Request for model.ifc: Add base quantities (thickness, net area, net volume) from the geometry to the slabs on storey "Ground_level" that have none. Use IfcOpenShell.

First a look at what the model holds.

```python
import ifcopenshell
import ifcopenshell.util.element
import ifcopenshell.util.unit

model = ifcopenshell.open("model.ifc")
print(model.schema)
for unit_type in ("LENGTHUNIT", "AREAUNIT", "VOLUMEUNIT"):
    print(unit_type, ifcopenshell.util.unit.calculate_unit_scale(model, unit_type))
storey = next(s for s in model.by_type("IfcBuildingStorey") if s.Name == "Ground_level")
slabs = [e for e in ifcopenshell.util.element.get_decomposition(storey) if e.is_a("IfcSlab")]
for e in sorted(slabs, key=lambda e: e.id()):
    print(e.id(), e.is_a(), e.Name, list(ifcopenshell.util.element.get_psets(e, qtos_only=True)), sep=" | ")
```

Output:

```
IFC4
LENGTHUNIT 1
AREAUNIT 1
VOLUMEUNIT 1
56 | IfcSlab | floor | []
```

```python
import ifcopenshell
import ifcopenshell.api.pset
import ifcopenshell.geom
import ifcopenshell.util.element
import ifcopenshell.util.shape
import ifcopenshell.util.unit

model = ifcopenshell.open("model.ifc")
unit_scale = ifcopenshell.util.unit.calculate_unit_scale(model)
area_scale = ifcopenshell.util.unit.calculate_unit_scale(model, "AREAUNIT")
volume_scale = ifcopenshell.util.unit.calculate_unit_scale(model, "VOLUMEUNIT")
settings = ifcopenshell.geom.settings()

storey = next(s for s in model.by_type("IfcBuildingStorey") if s.Name == "Ground_level")
slabs = [e for e in ifcopenshell.util.element.get_decomposition(storey) if e.is_a("IfcSlab")]

for e in sorted(slabs, key=lambda e: e.id()):
    if ifcopenshell.util.element.get_psets(e, qtos_only=True, should_inherit=False):
        continue
    # Geometry comes back in metres, in the element's own axes.
    shape = ifcopenshell.geom.create_shape(settings, e)
    values = {
        "Width": ifcopenshell.util.shape.get_z(shape.geometry) / unit_scale,
        "NetArea": ifcopenshell.util.shape.get_footprint_area(shape.geometry) / area_scale,
        "NetVolume": ifcopenshell.util.shape.get_volume(shape.geometry) / volume_scale,
    }
    qto = ifcopenshell.api.pset.add_qto(model, product=e, name="Qto_SlabBaseQuantities")
    ifcopenshell.api.pset.edit_qto(model, qto=qto, properties=values)
    print(e.id(), {k: round(v, 3) for k, v in values.items()})

model.write("model_v2.ifc")
```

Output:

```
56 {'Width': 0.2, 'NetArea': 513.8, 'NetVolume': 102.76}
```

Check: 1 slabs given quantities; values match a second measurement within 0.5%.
